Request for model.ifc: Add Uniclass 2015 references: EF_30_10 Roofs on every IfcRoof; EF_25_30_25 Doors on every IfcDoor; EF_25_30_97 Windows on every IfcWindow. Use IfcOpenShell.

First a look at what the model holds.

```python
import ifcopenshell

model = ifcopenshell.open("model.ifc")
print(model.schema)
print("classifications:", [c.Name for c in model.by_type("IfcClassification")])
for ifc_class in ("IfcDoor", "IfcRoof", "IfcStair", "IfcWall", "IfcWindow"):
    print(ifc_class, len(model.by_type(ifc_class)))
```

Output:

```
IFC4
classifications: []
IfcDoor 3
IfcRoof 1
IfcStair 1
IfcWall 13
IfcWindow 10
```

```python
import ifcopenshell
import ifcopenshell.api.classification

model = ifcopenshell.open("model.ifc")

system = ifcopenshell.api.classification.add_classification(model, classification="Uniclass 2015")

codes = {
    "IfcRoof": ("EF_30_10", "Roofs"),
    "IfcDoor": ("EF_25_30_25", "Doors"),
    "IfcWindow": ("EF_25_30_97", "Windows"),
}
for ifc_class, (code, name) in codes.items():
    products = model.by_type(ifc_class)
    ifcopenshell.api.classification.add_reference(
        model, products=products, classification=system, identification=code, name=name
    )
    print(code, len(products))

model.write("model_updated.ifc")
```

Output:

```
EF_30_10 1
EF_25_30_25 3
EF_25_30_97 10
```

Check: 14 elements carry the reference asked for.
